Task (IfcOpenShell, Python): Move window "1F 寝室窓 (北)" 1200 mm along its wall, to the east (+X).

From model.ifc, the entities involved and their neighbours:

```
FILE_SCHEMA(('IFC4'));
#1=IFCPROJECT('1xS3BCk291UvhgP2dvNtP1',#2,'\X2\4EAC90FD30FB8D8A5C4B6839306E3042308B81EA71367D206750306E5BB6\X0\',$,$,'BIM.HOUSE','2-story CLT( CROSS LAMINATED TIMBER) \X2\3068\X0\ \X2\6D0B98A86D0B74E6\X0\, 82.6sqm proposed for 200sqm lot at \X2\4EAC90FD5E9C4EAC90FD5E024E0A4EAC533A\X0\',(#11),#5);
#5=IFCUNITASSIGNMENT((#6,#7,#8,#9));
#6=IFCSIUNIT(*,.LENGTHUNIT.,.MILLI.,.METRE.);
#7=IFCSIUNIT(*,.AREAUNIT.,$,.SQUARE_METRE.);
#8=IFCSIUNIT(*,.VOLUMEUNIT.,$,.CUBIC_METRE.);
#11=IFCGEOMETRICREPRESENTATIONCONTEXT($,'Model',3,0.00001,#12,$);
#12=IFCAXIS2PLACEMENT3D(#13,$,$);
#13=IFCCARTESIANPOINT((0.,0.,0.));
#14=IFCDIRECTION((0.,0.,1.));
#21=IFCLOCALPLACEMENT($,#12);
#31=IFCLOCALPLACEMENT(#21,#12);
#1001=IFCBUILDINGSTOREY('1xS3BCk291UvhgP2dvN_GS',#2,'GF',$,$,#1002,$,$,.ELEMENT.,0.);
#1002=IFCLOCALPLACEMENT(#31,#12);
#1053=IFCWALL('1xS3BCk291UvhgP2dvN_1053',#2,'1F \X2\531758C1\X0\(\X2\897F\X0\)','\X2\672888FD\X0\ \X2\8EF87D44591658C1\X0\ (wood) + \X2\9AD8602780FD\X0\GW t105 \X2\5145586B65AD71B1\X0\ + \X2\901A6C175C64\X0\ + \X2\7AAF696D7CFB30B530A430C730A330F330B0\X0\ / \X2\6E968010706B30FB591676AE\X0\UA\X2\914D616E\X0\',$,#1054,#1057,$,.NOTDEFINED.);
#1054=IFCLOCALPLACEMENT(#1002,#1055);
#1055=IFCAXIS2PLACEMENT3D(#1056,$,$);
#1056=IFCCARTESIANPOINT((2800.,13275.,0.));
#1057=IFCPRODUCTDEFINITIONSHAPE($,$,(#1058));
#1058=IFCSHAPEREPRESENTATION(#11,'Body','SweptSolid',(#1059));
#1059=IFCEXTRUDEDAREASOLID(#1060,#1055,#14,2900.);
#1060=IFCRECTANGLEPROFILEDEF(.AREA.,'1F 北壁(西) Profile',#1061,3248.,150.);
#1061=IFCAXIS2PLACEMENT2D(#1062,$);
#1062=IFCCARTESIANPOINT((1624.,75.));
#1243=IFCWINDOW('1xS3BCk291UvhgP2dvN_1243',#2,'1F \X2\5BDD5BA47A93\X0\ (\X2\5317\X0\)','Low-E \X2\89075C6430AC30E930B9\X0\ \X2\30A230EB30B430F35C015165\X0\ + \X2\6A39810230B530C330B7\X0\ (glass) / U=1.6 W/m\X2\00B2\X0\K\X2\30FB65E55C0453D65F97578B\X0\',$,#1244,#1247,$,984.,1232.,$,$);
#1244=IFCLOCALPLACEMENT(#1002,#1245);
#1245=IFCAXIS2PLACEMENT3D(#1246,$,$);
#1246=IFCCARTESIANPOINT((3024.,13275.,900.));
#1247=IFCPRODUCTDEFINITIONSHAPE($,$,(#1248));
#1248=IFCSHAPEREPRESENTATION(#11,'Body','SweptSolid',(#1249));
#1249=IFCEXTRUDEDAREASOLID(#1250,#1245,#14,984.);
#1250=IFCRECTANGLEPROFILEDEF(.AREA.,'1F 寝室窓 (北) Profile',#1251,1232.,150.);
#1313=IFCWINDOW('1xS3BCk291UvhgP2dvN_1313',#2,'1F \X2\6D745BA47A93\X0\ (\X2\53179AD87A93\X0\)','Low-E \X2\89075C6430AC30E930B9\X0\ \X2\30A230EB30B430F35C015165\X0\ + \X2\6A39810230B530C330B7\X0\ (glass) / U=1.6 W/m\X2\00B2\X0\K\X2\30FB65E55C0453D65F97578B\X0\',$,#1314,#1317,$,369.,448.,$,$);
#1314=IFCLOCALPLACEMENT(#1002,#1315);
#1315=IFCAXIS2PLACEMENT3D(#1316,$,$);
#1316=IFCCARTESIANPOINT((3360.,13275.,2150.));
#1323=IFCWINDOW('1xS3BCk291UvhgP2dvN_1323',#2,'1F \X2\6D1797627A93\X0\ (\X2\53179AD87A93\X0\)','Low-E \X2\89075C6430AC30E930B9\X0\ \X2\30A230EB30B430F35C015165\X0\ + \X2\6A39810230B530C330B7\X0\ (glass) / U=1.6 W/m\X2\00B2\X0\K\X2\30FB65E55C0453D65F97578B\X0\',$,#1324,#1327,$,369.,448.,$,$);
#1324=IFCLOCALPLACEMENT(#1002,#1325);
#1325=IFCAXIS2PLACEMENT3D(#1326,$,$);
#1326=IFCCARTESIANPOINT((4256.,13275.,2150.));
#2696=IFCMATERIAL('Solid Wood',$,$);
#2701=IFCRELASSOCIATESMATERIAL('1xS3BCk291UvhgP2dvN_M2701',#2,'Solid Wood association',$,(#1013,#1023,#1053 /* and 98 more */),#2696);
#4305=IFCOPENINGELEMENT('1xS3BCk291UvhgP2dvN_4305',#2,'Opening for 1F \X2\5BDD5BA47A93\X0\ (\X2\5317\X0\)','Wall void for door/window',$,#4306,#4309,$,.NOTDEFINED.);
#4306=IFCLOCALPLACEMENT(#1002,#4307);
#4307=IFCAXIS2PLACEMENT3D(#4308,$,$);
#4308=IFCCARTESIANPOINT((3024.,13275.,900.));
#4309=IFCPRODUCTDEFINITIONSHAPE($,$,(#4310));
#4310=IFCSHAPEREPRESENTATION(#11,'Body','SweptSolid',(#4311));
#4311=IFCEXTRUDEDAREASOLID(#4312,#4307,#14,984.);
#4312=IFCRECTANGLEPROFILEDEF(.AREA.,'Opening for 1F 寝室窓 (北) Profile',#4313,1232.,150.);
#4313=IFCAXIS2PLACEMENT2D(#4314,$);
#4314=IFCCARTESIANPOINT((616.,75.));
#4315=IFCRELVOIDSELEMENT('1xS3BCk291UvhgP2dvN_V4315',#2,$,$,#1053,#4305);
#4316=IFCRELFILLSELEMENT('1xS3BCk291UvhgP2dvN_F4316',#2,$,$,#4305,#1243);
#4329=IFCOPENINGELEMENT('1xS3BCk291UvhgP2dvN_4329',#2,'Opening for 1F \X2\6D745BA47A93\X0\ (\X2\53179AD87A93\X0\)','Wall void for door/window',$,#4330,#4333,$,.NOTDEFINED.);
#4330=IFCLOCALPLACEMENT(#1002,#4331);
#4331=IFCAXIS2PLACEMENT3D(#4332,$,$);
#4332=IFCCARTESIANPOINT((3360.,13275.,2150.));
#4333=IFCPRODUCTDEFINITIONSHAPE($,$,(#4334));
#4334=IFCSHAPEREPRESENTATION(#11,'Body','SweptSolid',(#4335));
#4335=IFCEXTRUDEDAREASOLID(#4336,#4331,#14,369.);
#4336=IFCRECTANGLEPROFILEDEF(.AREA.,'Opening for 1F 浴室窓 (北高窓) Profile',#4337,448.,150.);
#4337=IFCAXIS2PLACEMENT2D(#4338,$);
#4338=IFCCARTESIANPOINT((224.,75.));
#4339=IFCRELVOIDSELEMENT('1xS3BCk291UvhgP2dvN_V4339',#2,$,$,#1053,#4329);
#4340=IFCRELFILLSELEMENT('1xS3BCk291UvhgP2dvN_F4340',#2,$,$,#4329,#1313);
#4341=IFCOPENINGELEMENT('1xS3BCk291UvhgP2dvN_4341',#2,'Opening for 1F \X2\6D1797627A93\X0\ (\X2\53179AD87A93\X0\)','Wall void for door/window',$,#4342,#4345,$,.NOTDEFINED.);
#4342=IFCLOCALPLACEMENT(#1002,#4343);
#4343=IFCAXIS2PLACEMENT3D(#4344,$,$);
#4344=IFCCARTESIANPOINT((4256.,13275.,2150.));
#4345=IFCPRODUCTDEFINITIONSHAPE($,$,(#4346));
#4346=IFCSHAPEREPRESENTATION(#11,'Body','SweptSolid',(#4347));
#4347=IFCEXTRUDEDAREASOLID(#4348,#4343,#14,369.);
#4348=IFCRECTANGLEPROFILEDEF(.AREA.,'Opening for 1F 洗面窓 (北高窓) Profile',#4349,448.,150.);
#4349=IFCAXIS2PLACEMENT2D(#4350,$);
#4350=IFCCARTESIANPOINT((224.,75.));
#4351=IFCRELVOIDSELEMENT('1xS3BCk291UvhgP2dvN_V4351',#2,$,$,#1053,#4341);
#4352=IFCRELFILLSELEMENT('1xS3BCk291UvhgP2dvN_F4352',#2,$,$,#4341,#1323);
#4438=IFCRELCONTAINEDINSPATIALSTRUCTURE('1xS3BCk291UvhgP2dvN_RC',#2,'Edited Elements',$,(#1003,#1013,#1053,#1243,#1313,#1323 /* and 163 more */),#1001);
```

```python
import ifcopenshell
import ifcopenshell.api.geometry
import ifcopenshell.util.placement
import ifcopenshell.util.unit

model = ifcopenshell.open("model.ifc")
unit_scale = ifcopenshell.util.unit.calculate_unit_scale(model)

window = model.by_guid("1xS3BCk291UvhgP2dvN_1243")
opening = window.FillsVoids[0].RelatingOpeningElement
wall = opening.VoidsElements[0].RelatingBuildingElement

wall_matrix = ifcopenshell.util.placement.get_local_placement(wall.ObjectPlacement)
shift = wall_matrix[:3, 0] * 1.2 / unit_scale
before = ifcopenshell.util.placement.get_local_placement(window.ObjectPlacement)[:3, 3].copy()

# The window is not placed relative to its opening, so move both.
for product in (opening, window):
    matrix = ifcopenshell.util.placement.get_local_placement(product.ObjectPlacement)
    matrix[:3, 3] += shift
    ifcopenshell.api.geometry.edit_object_placement(model, product=product, matrix=matrix, is_si=False)

after = ifcopenshell.util.placement.get_local_placement(window.ObjectPlacement)[:3, 3]
print("window moved by", (after - before).round(3) + 0.0)

model.write("model-out.ifc")
```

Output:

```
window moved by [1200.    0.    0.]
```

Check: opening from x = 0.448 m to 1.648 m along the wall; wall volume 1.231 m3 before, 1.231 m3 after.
